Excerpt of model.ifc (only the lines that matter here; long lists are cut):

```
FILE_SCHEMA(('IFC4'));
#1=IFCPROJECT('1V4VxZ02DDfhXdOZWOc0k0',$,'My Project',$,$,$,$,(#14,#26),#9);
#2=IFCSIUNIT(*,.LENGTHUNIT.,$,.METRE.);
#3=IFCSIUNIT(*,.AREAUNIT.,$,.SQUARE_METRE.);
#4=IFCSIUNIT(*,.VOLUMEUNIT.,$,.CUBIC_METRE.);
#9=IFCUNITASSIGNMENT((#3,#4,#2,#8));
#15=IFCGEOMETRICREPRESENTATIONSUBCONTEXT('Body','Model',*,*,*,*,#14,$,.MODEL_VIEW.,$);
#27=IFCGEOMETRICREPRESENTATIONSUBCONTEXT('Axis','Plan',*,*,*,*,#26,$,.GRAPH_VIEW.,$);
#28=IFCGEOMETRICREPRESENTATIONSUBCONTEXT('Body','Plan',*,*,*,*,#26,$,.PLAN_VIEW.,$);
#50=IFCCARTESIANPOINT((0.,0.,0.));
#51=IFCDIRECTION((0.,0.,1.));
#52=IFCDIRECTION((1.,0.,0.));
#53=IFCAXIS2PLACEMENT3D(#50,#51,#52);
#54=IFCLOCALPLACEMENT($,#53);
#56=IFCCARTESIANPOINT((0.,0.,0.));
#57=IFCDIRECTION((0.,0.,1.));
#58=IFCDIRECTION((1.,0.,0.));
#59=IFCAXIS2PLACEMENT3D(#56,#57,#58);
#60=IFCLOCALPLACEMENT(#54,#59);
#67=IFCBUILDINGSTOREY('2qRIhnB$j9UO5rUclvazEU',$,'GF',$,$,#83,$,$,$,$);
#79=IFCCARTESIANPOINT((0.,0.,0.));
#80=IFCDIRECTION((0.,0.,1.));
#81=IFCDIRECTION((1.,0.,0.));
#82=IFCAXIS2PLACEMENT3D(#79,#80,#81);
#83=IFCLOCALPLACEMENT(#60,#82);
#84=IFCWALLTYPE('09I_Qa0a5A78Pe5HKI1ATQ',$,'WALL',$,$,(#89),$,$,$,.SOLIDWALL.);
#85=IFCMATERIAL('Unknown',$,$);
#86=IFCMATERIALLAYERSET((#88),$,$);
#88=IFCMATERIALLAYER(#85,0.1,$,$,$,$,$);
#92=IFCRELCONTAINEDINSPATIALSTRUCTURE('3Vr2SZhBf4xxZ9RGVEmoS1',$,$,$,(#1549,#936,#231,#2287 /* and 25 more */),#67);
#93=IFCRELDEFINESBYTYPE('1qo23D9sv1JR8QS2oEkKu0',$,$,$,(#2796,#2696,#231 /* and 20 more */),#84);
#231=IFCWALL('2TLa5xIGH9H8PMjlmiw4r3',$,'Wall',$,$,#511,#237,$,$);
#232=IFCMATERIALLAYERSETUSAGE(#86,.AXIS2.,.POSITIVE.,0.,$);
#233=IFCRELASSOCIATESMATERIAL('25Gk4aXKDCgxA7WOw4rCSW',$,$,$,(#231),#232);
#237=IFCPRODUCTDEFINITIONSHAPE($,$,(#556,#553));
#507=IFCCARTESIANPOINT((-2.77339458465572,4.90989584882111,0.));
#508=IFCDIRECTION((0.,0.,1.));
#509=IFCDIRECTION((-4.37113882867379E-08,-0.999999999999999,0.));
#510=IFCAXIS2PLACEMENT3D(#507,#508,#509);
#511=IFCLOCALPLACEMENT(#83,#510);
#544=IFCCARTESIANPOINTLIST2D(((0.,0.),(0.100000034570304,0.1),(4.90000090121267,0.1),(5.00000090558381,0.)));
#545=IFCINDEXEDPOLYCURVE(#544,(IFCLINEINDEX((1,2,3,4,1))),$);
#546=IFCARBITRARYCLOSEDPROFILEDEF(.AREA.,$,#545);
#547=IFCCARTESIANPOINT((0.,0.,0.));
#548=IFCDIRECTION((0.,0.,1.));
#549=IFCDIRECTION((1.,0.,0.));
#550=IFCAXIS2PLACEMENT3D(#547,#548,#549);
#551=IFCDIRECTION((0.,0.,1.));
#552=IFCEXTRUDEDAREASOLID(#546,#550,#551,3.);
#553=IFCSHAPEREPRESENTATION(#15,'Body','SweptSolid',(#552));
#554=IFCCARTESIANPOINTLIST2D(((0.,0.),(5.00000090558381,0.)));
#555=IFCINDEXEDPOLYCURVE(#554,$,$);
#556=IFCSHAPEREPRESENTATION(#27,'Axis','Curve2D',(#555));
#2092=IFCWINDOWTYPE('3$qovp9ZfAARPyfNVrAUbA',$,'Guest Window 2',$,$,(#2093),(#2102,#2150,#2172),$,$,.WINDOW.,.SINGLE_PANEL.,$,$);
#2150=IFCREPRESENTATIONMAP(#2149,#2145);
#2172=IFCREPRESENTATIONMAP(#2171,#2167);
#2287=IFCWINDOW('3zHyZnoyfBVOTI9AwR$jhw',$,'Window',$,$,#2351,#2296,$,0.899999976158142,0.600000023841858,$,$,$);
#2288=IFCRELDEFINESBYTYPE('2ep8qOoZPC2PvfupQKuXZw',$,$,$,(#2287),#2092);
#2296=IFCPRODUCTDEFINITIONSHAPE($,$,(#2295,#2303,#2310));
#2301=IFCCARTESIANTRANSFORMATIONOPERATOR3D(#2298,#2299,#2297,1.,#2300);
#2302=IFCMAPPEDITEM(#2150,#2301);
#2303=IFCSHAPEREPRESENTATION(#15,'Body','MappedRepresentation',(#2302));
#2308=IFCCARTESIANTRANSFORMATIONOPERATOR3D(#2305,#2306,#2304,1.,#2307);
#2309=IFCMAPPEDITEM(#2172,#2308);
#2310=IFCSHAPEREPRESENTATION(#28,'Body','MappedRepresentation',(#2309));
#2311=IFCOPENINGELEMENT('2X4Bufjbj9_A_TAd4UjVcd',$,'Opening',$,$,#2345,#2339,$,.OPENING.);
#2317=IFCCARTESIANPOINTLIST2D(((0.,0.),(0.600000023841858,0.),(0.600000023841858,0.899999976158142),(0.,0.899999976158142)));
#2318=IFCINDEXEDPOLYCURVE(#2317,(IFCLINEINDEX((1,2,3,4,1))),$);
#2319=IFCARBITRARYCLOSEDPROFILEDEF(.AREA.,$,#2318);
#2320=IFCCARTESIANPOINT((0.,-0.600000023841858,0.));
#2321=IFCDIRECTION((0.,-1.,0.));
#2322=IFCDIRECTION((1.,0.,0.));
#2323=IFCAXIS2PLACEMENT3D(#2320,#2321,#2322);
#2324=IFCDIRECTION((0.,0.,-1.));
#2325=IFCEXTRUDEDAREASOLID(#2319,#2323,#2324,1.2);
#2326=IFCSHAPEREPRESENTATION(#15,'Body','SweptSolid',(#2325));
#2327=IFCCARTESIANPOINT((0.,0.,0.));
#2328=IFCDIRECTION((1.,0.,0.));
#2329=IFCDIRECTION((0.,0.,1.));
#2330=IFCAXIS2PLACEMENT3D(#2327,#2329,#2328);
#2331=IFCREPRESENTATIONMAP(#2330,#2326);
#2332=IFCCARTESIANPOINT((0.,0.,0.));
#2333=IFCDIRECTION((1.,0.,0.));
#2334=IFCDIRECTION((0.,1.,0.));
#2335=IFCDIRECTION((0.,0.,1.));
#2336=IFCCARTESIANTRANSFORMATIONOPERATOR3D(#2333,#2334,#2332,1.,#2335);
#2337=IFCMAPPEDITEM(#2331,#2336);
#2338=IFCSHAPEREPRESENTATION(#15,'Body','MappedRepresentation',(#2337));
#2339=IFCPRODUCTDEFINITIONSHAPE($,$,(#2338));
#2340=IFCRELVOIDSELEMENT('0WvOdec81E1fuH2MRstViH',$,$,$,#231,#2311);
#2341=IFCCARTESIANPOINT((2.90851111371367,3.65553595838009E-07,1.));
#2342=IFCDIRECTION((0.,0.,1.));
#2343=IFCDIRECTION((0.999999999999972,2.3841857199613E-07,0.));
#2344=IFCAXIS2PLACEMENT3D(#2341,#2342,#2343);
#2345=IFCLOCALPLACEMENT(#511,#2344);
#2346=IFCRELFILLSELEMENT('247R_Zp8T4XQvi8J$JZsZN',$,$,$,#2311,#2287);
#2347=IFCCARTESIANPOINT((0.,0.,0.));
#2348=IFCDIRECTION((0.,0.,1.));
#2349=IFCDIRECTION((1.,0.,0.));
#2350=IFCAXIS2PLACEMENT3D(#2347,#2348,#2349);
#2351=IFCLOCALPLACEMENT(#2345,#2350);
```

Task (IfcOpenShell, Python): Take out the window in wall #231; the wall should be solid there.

```python
import ifcopenshell
import ifcopenshell.api.feature
import ifcopenshell.api.root
import ifcopenshell.geom
import ifcopenshell.util.shape

model = ifcopenshell.open("model.ifc")
settings = ifcopenshell.geom.settings()


def volume(element):
    """Net volume in cubic metres, openings subtracted."""
    shape = ifcopenshell.geom.create_shape(settings, element)
    return ifcopenshell.util.shape.get_volume(shape.geometry)


window = model.by_id(2287)
opening = window.FillsVoids[0].RelatingOpeningElement
wall = opening.VoidsElements[0].RelatingBuildingElement
before = volume(wall)

ifcopenshell.api.root.remove_product(model, product=window)
ifcopenshell.api.feature.remove_feature(model, feature=opening)

after = volume(wall)

print(f"wall volume {before:.3f} -> {after:.3f} m3")

model.write("model_v2.ifc")
```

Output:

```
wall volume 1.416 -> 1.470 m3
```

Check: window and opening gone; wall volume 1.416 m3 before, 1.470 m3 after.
